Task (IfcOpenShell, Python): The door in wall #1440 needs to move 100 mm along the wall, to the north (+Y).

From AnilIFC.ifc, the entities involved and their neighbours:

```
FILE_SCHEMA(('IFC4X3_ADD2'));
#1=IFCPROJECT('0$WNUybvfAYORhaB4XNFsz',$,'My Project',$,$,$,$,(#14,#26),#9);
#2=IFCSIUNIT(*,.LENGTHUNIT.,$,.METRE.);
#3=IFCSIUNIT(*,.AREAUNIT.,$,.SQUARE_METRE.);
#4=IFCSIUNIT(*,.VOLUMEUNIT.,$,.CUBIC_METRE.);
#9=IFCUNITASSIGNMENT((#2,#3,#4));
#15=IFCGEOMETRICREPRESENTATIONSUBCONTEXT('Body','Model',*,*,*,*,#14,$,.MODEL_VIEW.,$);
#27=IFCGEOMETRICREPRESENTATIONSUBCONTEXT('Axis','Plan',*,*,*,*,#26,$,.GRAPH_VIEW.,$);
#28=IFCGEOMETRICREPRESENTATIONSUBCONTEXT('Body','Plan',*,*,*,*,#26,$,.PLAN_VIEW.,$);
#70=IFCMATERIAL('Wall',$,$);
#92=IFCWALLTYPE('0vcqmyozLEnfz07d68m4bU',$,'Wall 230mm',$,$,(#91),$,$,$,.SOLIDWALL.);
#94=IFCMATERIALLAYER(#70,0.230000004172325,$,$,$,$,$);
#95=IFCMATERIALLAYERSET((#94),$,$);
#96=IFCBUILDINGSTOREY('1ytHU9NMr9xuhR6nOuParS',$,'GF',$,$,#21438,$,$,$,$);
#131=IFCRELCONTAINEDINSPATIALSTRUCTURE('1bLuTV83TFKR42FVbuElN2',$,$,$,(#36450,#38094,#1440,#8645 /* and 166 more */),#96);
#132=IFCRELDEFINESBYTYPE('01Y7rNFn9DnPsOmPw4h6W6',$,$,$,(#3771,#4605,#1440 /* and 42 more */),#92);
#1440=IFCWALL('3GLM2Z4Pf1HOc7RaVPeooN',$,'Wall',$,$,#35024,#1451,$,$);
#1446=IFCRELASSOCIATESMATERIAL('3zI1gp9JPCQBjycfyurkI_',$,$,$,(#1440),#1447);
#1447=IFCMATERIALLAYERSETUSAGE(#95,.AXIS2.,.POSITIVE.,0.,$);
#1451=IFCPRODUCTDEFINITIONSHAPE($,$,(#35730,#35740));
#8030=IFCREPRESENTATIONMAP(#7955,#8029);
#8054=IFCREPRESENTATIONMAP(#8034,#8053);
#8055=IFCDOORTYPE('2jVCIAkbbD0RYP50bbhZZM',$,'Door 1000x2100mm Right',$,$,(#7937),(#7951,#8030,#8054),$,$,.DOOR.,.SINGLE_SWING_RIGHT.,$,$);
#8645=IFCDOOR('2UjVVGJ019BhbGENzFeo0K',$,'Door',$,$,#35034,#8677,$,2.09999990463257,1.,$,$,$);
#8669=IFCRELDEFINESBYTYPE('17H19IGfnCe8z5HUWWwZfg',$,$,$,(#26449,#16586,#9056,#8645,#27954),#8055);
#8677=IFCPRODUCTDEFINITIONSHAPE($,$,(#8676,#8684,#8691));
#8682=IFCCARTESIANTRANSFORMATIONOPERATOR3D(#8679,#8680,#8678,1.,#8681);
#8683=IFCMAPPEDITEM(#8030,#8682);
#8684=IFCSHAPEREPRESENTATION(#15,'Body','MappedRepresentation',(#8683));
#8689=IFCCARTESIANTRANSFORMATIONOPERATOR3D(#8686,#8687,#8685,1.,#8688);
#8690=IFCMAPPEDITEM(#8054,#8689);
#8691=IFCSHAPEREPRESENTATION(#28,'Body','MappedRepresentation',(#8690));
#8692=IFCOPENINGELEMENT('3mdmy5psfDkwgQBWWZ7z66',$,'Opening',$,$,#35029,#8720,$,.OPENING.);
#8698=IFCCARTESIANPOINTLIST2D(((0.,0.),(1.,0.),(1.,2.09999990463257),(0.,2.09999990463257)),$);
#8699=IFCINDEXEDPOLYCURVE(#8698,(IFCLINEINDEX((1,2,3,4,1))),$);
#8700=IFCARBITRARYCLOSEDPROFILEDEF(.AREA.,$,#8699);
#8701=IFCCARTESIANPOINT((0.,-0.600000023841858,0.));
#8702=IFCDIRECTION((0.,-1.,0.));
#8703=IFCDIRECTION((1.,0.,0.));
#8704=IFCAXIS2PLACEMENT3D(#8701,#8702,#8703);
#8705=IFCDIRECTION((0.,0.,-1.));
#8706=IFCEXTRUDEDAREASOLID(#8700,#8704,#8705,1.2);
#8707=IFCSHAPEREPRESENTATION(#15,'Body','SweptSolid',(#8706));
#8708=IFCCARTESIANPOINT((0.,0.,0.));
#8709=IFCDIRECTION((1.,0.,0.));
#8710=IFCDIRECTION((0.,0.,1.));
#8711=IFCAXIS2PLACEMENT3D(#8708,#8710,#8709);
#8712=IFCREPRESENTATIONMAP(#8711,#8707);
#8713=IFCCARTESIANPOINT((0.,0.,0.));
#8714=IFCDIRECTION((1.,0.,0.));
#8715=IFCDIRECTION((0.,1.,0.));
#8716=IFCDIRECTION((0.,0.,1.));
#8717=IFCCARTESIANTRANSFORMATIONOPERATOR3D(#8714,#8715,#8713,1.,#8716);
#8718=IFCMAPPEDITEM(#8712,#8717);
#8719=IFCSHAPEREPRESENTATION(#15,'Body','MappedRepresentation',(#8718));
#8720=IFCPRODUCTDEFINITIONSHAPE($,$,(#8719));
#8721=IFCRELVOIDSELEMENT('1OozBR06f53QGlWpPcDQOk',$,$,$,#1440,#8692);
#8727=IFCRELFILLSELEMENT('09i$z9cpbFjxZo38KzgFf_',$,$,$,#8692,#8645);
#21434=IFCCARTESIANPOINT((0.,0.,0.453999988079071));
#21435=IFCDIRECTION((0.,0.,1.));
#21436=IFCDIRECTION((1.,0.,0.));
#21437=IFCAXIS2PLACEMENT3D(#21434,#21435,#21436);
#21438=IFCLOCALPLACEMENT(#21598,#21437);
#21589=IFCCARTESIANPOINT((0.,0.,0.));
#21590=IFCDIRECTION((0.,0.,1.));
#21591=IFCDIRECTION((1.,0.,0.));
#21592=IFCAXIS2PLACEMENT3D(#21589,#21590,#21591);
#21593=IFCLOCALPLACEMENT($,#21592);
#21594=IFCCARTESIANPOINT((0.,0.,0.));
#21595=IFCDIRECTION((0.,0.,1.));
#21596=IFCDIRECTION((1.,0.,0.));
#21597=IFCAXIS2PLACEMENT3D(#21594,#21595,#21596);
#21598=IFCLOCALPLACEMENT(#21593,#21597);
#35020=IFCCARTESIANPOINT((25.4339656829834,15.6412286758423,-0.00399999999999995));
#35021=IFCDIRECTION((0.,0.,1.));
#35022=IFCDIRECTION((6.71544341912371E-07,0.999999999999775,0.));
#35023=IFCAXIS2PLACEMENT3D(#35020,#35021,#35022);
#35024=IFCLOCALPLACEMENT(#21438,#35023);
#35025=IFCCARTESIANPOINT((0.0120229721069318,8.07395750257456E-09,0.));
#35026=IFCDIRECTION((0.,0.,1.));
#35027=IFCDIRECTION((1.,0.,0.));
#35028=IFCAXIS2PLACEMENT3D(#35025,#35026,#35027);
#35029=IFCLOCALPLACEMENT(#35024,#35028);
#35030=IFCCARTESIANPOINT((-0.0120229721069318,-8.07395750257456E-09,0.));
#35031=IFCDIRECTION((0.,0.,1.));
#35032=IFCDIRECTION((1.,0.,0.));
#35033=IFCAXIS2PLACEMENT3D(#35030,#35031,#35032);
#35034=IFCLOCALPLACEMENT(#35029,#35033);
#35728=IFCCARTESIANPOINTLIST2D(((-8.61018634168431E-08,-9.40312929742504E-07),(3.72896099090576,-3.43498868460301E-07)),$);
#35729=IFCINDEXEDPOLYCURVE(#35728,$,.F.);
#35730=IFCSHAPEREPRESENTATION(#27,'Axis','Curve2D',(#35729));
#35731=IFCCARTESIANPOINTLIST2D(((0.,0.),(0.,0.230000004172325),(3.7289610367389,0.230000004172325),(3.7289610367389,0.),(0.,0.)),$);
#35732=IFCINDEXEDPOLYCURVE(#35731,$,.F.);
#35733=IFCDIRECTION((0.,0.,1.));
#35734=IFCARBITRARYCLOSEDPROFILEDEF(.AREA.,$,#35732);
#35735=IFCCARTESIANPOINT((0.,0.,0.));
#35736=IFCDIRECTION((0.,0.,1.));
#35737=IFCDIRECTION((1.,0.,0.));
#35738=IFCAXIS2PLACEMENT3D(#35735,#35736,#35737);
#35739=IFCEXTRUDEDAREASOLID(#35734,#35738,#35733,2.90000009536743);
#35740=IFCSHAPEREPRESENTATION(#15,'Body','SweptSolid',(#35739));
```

```python
import ifcopenshell
import ifcopenshell.api.geometry
import ifcopenshell.util.placement

model = ifcopenshell.open("AnilIFC.ifc")

door = model.by_guid("2UjVVGJ019BhbGENzFeo0K")
opening = door.FillsVoids[0].RelatingOpeningElement
wall = opening.VoidsElements[0].RelatingBuildingElement

wall_matrix = ifcopenshell.util.placement.get_local_placement(wall.ObjectPlacement)
shift = wall_matrix[:3, 0] * 0.1
before = ifcopenshell.util.placement.get_local_placement(door.ObjectPlacement)[:3, 3].copy()

# The door is placed relative to its opening, so it follows when the opening moves.
matrix = ifcopenshell.util.placement.get_local_placement(opening.ObjectPlacement)
matrix[:3, 3] += shift
ifcopenshell.api.geometry.edit_object_placement(
    model, product=opening, matrix=matrix, is_si=False, should_transform_children=True
)

after = ifcopenshell.util.placement.get_local_placement(door.ObjectPlacement)[:3, 3]
print("door moved by", (after - before).round(3) + 0.0)

model.write("AnilIFC-out.ifc")
```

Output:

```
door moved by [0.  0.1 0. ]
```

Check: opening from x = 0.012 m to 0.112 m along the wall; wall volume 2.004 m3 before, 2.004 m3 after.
